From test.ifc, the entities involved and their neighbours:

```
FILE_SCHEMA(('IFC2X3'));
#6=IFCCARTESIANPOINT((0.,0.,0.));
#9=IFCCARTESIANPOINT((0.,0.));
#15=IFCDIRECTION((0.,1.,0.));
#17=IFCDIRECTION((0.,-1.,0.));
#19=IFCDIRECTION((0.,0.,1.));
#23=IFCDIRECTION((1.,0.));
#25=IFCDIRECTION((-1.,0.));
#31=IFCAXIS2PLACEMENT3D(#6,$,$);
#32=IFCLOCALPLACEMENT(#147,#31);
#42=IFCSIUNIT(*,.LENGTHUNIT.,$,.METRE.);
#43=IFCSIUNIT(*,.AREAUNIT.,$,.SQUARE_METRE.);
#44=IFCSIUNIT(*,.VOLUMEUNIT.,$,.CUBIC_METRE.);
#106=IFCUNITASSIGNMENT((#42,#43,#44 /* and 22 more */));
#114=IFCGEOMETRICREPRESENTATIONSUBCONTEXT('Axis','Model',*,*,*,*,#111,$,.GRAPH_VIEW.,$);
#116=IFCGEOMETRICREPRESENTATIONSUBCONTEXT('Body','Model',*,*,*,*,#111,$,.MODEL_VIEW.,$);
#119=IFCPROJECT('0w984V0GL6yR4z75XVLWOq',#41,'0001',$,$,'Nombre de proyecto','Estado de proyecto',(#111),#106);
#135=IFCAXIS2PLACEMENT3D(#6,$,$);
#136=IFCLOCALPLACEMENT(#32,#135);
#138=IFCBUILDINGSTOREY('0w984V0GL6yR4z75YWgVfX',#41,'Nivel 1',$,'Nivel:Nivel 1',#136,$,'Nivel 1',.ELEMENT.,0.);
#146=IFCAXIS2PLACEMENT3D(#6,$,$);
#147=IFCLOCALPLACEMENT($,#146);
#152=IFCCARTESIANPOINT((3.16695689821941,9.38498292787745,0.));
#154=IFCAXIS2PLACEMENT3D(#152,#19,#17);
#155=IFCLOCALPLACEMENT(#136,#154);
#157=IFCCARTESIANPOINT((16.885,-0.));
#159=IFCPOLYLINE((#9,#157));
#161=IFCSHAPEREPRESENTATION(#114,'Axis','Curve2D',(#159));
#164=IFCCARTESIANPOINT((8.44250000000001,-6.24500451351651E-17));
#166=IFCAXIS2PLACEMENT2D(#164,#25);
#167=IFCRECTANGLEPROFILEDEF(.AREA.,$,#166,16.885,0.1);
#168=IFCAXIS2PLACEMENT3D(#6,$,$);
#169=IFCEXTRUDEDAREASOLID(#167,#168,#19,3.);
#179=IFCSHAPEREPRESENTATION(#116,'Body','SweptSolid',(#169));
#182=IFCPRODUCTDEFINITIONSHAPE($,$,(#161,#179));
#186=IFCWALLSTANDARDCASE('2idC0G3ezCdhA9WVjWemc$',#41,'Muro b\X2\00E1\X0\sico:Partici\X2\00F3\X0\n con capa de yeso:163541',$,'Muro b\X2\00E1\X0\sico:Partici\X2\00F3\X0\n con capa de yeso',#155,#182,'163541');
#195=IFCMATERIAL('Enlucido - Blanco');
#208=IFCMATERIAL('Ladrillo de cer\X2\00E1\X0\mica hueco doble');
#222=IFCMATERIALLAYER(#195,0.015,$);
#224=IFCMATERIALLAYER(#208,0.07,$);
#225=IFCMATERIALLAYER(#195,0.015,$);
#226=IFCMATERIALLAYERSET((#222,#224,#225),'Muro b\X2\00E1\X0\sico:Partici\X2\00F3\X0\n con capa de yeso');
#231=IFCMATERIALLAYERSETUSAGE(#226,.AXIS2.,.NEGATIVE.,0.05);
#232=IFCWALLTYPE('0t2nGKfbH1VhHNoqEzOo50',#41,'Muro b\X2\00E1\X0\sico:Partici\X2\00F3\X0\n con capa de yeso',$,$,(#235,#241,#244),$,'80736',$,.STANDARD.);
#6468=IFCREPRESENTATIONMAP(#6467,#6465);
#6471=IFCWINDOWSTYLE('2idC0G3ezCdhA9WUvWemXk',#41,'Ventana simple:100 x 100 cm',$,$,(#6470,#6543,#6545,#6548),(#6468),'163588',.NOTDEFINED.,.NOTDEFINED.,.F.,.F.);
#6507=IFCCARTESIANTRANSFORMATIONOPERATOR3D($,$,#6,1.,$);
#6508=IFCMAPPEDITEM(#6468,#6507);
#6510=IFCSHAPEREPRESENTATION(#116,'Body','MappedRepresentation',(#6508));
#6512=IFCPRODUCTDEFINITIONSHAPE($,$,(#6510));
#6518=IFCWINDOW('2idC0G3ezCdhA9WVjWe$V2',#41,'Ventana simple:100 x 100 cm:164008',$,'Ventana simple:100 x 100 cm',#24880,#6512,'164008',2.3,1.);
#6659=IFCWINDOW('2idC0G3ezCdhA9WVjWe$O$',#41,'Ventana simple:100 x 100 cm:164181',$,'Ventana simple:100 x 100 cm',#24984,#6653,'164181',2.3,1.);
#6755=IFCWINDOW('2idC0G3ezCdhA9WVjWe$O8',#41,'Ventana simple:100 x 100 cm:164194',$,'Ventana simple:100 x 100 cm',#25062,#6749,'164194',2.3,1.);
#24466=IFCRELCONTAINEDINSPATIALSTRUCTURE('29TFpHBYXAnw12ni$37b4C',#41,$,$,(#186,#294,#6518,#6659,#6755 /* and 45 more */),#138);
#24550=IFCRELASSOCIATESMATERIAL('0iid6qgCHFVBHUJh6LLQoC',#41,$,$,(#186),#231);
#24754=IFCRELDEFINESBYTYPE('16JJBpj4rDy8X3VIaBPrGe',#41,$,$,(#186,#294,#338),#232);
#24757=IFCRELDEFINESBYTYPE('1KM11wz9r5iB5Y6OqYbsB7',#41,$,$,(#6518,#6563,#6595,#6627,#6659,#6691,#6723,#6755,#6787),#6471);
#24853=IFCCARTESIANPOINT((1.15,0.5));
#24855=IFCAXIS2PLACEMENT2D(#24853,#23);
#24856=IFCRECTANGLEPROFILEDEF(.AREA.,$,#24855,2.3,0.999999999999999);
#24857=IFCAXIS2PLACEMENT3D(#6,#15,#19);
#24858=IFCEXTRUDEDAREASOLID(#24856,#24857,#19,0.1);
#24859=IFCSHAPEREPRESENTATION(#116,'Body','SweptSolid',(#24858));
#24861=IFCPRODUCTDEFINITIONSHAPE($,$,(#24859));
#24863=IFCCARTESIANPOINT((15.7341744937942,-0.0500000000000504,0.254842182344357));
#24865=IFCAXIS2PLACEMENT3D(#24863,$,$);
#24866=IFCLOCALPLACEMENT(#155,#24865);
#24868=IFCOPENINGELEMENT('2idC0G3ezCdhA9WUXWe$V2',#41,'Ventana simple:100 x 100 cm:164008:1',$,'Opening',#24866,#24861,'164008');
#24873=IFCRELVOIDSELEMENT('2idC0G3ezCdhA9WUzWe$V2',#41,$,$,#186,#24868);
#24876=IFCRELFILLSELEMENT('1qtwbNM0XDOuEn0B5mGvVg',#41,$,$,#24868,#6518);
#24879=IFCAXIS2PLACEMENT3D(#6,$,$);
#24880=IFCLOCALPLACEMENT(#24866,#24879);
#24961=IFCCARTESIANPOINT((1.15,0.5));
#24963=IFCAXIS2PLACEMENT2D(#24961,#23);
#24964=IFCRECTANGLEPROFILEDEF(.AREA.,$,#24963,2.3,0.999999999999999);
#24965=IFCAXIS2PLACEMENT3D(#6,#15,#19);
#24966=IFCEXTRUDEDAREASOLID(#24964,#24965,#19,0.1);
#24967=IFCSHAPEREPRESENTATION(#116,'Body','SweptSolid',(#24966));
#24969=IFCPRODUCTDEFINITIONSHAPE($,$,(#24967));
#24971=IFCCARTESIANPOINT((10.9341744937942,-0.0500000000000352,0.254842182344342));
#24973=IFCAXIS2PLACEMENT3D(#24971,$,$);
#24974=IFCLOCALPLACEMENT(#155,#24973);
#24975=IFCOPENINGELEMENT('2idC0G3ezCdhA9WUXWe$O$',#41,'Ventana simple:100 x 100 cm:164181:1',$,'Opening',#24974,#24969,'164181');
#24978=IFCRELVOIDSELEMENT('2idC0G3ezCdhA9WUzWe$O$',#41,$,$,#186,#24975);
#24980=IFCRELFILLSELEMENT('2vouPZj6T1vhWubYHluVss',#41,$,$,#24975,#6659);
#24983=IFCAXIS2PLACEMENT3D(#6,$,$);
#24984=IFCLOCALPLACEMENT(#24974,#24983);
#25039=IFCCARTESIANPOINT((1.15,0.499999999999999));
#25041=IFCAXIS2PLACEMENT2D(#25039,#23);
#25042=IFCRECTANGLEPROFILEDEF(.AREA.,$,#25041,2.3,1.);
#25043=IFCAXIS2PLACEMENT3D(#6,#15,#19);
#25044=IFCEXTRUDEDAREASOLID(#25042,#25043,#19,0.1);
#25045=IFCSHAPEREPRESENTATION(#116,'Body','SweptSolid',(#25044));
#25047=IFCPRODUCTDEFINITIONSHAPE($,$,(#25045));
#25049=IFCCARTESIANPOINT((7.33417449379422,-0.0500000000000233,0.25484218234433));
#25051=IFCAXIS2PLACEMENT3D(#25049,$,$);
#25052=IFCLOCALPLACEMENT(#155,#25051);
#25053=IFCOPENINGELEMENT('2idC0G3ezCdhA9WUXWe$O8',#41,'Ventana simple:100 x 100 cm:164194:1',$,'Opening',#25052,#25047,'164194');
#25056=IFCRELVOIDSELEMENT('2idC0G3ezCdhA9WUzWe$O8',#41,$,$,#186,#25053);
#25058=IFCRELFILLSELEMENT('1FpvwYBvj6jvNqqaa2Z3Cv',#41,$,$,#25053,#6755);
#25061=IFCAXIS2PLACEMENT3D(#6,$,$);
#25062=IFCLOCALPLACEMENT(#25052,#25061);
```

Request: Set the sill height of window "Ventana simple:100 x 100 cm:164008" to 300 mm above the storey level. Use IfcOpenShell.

```python
import numpy as np
import ifcopenshell
import ifcopenshell.api.geometry
import ifcopenshell.geom
import ifcopenshell.util.element
import ifcopenshell.util.placement
import ifcopenshell.util.shape
import ifcopenshell.util.unit

model = ifcopenshell.open("test.ifc")
unit_scale = ifcopenshell.util.unit.calculate_unit_scale(model)

window = model.by_guid("2idC0G3ezCdhA9WVjWe$V2")
opening = window.FillsVoids[0].RelatingOpeningElement
storey = ifcopenshell.util.element.get_container(window, ifc_class="IfcBuildingStorey")
level = ifcopenshell.util.placement.get_local_placement(storey.ObjectPlacement)[2, 3]

# The opening's origin need not be at the sill, so measure its lowest point.
shape = ifcopenshell.geom.create_shape(ifcopenshell.geom.settings(), opening)
bottom = ifcopenshell.util.shape.get_shape_bottom_elevation(shape, shape.geometry) / unit_scale
dz = level + 0.3 / unit_scale - bottom

shift = np.array([0.0, 0.0, dz])
# The window is placed relative to its opening, so it follows when the opening moves.
matrix = ifcopenshell.util.placement.get_local_placement(opening.ObjectPlacement)
matrix[:3, 3] += shift
ifcopenshell.api.geometry.edit_object_placement(
    model, product=opening, matrix=matrix, is_si=False, should_transform_children=True
)

print(f"moved by {dz * unit_scale:+.3f} m")

model.write("test_edited.ifc")
```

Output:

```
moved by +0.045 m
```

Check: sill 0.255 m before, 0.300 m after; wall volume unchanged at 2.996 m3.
